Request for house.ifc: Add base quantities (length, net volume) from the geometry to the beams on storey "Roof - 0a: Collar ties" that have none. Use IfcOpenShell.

First a look at what the model holds.

```python
import ifcopenshell
import ifcopenshell.util.element
import ifcopenshell.util.unit

model = ifcopenshell.open("house.ifc")
print(model.schema)
for unit_type in ("LENGTHUNIT", "AREAUNIT", "VOLUMEUNIT"):
    print(unit_type, ifcopenshell.util.unit.calculate_unit_scale(model, unit_type))
storey = next(s for s in model.by_type("IfcBuildingStorey") if s.Name == "Roof - 0a: Collar ties")
beams = [e for e in ifcopenshell.util.element.get_decomposition(storey) if e.is_a("IfcBeam")]
for e in sorted(beams, key=lambda e: e.id()):
    print(e.id(), e.is_a(), e.Name, list(ifcopenshell.util.element.get_psets(e, qtos_only=True)), sep=" | ")
```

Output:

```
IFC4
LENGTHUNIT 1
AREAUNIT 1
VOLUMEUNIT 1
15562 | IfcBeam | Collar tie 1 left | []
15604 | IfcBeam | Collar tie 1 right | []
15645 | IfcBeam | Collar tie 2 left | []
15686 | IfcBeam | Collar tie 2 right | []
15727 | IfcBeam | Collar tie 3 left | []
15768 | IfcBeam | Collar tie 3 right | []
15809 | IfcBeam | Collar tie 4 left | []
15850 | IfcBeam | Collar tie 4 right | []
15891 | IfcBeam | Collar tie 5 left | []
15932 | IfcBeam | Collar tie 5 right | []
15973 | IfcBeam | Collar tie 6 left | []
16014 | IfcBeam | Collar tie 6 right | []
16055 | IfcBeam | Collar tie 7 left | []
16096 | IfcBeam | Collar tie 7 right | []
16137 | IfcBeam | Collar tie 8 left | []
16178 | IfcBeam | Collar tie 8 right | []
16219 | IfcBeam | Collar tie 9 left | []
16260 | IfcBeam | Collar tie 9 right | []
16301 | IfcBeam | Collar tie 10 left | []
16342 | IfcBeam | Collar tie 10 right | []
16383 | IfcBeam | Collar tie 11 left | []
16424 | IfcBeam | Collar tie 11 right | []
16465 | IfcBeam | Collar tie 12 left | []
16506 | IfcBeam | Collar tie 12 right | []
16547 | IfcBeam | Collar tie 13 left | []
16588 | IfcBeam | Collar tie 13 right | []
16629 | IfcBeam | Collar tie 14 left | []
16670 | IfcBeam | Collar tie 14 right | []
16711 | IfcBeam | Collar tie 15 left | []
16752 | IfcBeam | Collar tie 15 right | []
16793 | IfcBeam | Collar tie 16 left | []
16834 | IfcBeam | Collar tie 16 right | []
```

```python
import ifcopenshell
import ifcopenshell.api.pset
import ifcopenshell.geom
import ifcopenshell.util.element
import ifcopenshell.util.shape
import ifcopenshell.util.unit

model = ifcopenshell.open("house.ifc")
unit_scale = ifcopenshell.util.unit.calculate_unit_scale(model)
volume_scale = ifcopenshell.util.unit.calculate_unit_scale(model, "VOLUMEUNIT")
settings = ifcopenshell.geom.settings()

storey = next(s for s in model.by_type("IfcBuildingStorey") if s.Name == "Roof - 0a: Collar ties")
beams = [e for e in ifcopenshell.util.element.get_decomposition(storey) if e.is_a("IfcBeam")]

for e in sorted(beams, key=lambda e: e.id()):
    if ifcopenshell.util.element.get_psets(e, qtos_only=True, should_inherit=False):
        continue
    # Geometry comes back in metres, in the element's own axes.
    shape = ifcopenshell.geom.create_shape(settings, e)
    values = {
        "Length": ifcopenshell.util.shape.get_max_xyz(shape.geometry) / unit_scale,
        "NetVolume": ifcopenshell.util.shape.get_volume(shape.geometry) / volume_scale,
    }
    qto = ifcopenshell.api.pset.add_qto(model, product=e, name="Qto_BeamBaseQuantities")
    ifcopenshell.api.pset.edit_qto(model, qto=qto, properties=values)
    print(e.id(), {k: round(v, 3) for k, v in values.items()})

model.write("house_edited.ifc")
```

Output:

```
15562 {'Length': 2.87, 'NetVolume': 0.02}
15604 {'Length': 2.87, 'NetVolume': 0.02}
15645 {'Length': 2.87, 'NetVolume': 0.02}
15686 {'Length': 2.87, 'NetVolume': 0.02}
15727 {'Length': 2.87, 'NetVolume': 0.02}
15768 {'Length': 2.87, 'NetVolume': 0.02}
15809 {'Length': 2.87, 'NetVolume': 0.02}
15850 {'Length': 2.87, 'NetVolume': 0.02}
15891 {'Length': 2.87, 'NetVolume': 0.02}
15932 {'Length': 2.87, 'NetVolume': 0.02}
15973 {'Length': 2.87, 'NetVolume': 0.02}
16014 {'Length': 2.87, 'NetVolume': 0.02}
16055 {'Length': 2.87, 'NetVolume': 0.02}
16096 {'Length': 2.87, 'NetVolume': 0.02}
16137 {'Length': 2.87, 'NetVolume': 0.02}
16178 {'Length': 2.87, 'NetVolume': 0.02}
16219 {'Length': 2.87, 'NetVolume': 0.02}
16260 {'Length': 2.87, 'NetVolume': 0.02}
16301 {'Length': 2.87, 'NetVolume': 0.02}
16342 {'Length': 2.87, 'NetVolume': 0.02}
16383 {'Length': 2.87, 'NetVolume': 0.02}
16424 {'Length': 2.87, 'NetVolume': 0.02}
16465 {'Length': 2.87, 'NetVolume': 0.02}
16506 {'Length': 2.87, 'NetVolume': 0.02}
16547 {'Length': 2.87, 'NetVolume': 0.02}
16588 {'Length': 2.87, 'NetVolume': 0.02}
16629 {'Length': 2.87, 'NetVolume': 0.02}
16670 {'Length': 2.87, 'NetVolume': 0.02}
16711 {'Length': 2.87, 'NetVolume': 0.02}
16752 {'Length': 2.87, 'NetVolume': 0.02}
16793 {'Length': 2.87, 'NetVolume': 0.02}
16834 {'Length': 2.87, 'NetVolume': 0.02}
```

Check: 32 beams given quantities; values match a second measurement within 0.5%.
